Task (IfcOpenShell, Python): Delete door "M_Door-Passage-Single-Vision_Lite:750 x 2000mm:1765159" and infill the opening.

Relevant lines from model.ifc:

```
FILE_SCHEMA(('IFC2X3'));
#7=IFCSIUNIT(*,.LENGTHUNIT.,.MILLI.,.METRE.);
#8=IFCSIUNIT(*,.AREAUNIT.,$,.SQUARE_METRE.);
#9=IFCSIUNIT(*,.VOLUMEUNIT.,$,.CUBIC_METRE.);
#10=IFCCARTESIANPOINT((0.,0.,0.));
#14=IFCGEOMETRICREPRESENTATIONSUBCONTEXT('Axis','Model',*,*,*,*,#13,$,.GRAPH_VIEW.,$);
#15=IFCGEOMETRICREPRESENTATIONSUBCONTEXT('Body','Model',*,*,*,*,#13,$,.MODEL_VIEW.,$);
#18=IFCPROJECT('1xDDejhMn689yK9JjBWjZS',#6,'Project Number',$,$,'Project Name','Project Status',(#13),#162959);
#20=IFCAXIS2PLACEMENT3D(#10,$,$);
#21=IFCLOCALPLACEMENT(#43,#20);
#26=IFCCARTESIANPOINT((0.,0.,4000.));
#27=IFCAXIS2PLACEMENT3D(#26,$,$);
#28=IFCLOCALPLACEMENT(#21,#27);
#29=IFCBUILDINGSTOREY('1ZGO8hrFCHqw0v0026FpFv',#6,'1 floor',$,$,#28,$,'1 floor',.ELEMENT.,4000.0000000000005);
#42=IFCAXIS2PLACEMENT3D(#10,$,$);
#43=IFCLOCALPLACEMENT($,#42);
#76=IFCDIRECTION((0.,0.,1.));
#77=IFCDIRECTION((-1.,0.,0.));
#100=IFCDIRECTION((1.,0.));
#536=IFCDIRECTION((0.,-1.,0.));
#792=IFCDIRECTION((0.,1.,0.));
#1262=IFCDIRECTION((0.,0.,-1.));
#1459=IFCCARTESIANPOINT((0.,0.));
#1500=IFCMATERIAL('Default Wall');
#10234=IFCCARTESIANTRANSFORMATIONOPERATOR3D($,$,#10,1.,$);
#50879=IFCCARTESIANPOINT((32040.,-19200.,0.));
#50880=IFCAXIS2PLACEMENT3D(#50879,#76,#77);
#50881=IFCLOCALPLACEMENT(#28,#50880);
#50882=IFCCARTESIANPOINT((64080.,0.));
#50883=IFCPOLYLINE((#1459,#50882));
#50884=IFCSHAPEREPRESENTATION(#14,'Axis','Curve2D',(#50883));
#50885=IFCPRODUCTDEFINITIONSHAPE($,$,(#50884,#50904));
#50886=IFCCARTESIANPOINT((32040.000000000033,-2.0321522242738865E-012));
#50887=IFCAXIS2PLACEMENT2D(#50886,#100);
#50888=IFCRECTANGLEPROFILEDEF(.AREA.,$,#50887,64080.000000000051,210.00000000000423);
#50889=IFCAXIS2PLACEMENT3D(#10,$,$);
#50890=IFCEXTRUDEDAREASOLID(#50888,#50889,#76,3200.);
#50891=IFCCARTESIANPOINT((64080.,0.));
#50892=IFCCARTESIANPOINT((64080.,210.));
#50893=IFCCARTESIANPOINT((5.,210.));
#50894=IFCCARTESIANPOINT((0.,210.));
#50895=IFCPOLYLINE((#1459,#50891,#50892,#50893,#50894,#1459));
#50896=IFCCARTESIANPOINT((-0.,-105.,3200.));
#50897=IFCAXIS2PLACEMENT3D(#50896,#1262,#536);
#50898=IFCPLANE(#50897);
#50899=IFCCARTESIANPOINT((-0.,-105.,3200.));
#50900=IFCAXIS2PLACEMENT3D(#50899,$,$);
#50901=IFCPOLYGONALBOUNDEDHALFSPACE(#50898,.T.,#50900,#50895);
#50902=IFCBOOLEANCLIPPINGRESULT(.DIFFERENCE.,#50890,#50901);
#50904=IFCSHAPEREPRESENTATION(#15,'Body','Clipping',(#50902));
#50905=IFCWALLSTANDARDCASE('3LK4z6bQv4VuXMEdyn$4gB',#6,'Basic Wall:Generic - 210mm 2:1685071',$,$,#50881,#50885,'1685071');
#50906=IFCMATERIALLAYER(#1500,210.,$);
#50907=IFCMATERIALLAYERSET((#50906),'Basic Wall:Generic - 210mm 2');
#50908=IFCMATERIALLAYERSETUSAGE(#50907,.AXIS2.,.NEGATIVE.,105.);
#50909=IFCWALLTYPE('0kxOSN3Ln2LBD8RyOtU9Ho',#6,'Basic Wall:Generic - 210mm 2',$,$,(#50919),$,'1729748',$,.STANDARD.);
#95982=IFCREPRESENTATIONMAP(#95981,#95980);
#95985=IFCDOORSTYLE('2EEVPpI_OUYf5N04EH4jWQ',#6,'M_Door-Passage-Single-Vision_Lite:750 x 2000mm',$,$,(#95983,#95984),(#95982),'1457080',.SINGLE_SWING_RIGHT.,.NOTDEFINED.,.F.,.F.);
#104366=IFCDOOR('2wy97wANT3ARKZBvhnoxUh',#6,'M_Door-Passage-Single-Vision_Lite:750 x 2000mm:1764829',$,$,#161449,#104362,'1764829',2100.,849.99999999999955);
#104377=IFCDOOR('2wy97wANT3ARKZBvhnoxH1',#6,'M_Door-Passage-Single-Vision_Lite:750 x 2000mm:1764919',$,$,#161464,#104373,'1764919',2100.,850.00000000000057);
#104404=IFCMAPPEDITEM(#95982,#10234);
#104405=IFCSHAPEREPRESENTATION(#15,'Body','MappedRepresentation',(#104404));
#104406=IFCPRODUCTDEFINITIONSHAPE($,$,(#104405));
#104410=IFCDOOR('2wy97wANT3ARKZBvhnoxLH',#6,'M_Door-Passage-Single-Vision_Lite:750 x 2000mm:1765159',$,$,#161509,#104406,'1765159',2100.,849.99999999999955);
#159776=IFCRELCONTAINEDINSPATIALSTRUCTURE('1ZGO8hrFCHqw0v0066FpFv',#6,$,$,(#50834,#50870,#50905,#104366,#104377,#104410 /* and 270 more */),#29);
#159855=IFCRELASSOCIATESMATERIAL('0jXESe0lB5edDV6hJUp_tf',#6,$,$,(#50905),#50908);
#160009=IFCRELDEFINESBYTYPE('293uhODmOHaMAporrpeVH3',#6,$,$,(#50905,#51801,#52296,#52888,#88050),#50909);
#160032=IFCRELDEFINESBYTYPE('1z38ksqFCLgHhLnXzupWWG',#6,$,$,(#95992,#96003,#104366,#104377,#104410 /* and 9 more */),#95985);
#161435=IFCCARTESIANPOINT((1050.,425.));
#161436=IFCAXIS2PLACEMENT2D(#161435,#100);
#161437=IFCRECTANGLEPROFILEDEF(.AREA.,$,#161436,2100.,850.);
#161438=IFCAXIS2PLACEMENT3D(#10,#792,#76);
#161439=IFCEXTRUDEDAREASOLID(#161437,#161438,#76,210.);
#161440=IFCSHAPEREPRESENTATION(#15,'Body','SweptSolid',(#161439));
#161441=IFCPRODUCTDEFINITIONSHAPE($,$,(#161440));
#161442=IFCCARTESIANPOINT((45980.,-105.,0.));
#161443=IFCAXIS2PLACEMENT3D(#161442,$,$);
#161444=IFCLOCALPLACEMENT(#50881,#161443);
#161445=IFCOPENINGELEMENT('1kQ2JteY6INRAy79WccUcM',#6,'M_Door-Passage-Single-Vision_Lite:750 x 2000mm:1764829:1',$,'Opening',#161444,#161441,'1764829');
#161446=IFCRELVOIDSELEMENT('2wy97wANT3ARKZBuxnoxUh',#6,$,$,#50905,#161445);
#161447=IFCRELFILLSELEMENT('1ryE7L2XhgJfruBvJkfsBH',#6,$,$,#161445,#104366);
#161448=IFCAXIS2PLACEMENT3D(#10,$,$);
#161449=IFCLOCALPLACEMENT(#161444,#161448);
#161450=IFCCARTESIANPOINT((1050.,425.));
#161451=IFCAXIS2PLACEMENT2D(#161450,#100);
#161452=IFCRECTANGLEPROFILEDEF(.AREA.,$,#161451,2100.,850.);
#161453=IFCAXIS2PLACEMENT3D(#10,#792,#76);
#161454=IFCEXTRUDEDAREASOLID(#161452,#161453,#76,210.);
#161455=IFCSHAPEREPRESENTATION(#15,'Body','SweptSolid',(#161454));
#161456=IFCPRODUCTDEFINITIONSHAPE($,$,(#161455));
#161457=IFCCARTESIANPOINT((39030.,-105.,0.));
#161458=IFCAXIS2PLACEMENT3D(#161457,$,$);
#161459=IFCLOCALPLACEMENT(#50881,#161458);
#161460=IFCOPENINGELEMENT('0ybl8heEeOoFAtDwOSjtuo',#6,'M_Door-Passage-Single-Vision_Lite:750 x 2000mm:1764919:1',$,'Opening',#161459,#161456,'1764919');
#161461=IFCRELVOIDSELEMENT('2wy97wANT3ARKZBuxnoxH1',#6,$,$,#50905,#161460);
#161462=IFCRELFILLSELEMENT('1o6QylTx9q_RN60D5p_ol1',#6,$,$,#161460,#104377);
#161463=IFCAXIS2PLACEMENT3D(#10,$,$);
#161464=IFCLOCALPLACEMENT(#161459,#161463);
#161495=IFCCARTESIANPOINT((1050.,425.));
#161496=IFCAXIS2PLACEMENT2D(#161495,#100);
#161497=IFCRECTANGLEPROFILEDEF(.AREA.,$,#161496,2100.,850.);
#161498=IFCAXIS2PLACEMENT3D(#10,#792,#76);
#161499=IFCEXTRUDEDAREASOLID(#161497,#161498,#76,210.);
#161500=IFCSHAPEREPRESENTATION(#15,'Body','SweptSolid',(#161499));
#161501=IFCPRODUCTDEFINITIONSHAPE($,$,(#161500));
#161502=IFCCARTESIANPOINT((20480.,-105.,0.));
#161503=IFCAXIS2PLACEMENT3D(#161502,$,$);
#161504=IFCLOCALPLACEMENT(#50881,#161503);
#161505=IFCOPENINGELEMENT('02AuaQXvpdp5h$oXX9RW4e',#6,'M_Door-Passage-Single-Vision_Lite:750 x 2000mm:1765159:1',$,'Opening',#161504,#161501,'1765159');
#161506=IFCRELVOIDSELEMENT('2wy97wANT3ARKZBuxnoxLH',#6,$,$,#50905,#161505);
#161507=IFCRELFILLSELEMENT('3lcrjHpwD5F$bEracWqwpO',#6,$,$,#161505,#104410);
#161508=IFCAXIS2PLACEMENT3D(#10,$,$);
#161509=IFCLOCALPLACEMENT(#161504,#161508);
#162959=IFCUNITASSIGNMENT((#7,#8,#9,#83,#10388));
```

```python
import ifcopenshell
import ifcopenshell.api.feature
import ifcopenshell.api.root
import ifcopenshell.geom
import ifcopenshell.util.shape

model = ifcopenshell.open("model.ifc")
settings = ifcopenshell.geom.settings()


def volume(element):
    """Net volume in cubic metres, openings subtracted."""
    shape = ifcopenshell.geom.create_shape(settings, element)
    return ifcopenshell.util.shape.get_volume(shape.geometry)


door = model.by_guid("2wy97wANT3ARKZBvhnoxLH")
opening = door.FillsVoids[0].RelatingOpeningElement
wall = opening.VoidsElements[0].RelatingBuildingElement
before = volume(wall)

ifcopenshell.api.root.remove_product(model, product=door)
ifcopenshell.api.feature.remove_feature(model, feature=opening)

after = volume(wall)

print(f"wall volume {before:.3f} -> {after:.3f} m3")

model.write("model_edited.ifc")
```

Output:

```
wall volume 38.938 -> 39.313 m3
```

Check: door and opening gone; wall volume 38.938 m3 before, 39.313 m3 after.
